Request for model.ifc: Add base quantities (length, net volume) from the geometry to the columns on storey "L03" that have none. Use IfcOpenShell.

First a look at what the model holds.

```python
import ifcopenshell
import ifcopenshell.util.element
import ifcopenshell.util.unit

model = ifcopenshell.open("model.ifc")
print(model.schema)
for unit_type in ("LENGTHUNIT", "AREAUNIT", "VOLUMEUNIT"):
    print(unit_type, ifcopenshell.util.unit.calculate_unit_scale(model, unit_type))
storey = next(s for s in model.by_type("IfcBuildingStorey") if s.Name == "L03")
columns = [e for e in ifcopenshell.util.element.get_decomposition(storey) if e.is_a("IfcColumn")]
for e in sorted(columns, key=lambda e: e.id()):
    print(e.id(), e.is_a(), e.Name, list(ifcopenshell.util.element.get_psets(e, qtos_only=True)), sep=" | ")
```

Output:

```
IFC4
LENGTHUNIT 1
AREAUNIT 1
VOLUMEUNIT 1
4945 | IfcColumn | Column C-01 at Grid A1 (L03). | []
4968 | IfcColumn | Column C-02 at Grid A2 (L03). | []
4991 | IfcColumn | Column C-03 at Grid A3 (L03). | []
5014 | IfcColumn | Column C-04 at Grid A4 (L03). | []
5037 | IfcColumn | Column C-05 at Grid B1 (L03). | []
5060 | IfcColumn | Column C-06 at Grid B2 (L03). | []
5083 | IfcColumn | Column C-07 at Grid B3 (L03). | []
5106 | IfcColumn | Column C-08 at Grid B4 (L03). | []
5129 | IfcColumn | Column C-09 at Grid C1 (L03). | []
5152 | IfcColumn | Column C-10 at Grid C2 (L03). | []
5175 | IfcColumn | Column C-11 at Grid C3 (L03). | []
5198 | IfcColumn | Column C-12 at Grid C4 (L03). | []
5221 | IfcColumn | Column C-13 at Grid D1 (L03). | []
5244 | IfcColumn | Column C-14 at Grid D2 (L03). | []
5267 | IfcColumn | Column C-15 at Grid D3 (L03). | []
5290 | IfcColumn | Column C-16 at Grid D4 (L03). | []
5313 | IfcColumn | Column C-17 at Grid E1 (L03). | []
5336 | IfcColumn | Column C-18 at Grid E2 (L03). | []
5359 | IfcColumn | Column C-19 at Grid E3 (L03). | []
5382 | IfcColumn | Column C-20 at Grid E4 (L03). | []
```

```python
import ifcopenshell
import ifcopenshell.api.pset
import ifcopenshell.geom
import ifcopenshell.util.element
import ifcopenshell.util.shape
import ifcopenshell.util.unit

model = ifcopenshell.open("model.ifc")
unit_scale = ifcopenshell.util.unit.calculate_unit_scale(model)
volume_scale = ifcopenshell.util.unit.calculate_unit_scale(model, "VOLUMEUNIT")
settings = ifcopenshell.geom.settings()

storey = next(s for s in model.by_type("IfcBuildingStorey") if s.Name == "L03")
columns = [e for e in ifcopenshell.util.element.get_decomposition(storey) if e.is_a("IfcColumn")]

for e in sorted(columns, key=lambda e: e.id()):
    if ifcopenshell.util.element.get_psets(e, qtos_only=True, should_inherit=False):
        continue
    # Geometry comes back in metres, in the element's own axes.
    shape = ifcopenshell.geom.create_shape(settings, e)
    values = {
        "Length": ifcopenshell.util.shape.get_z(shape.geometry) / unit_scale,
        "NetVolume": ifcopenshell.util.shape.get_volume(shape.geometry) / volume_scale,
    }
    qto = ifcopenshell.api.pset.add_qto(model, product=e, name="Qto_ColumnBaseQuantities")
    ifcopenshell.api.pset.edit_qto(model, qto=qto, properties=values)
    print(e.id(), {k: round(v, 3) for k, v in values.items()})

model.write("model_updated.ifc")
```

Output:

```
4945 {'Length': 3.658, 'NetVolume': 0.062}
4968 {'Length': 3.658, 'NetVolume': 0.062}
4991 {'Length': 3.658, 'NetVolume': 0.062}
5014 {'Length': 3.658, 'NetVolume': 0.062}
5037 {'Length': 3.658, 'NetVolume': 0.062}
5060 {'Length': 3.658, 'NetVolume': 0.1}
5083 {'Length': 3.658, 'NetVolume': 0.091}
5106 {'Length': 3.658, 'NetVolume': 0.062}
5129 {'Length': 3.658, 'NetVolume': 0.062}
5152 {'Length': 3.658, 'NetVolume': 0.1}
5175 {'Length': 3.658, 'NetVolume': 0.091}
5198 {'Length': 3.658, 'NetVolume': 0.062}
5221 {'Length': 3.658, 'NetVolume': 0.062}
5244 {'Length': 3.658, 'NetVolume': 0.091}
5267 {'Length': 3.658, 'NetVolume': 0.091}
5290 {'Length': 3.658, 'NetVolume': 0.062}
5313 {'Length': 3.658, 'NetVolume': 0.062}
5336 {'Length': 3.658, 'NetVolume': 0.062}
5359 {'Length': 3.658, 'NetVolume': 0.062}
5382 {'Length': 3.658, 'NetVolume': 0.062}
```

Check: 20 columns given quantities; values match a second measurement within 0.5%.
